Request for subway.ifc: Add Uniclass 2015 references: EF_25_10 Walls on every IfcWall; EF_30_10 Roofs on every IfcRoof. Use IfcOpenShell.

First a look at what the model holds.

```python
import ifcopenshell

model = ifcopenshell.open("subway.ifc")
print(model.schema)
print("classifications:", [c.Name for c in model.by_type("IfcClassification")])
for ifc_class in ("IfcDoor", "IfcRoof", "IfcStair", "IfcWall", "IfcWindow"):
    print(ifc_class, len(model.by_type(ifc_class)))
```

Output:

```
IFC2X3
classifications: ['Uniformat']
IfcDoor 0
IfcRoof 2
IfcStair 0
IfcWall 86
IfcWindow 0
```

```python
import ifcopenshell
import ifcopenshell.api.classification

model = ifcopenshell.open("subway.ifc")

# IFC2X3 requires Source and Edition and has no link from the project to the system.
system = model.create_entity("IfcClassification", Source="NBS", Edition="2015", Name="Uniclass 2015")

codes = {
    "IfcWall": ("EF_25_10", "Walls"),
    "IfcRoof": ("EF_30_10", "Roofs"),
}
for ifc_class, (code, name) in codes.items():
    products = model.by_type(ifc_class)
    ifcopenshell.api.classification.add_reference(
        model, products=products, classification=system, identification=code, name=name
    )
    print(code, len(products))

model.write("subway_v2.ifc")
```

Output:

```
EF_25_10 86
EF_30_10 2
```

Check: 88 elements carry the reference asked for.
